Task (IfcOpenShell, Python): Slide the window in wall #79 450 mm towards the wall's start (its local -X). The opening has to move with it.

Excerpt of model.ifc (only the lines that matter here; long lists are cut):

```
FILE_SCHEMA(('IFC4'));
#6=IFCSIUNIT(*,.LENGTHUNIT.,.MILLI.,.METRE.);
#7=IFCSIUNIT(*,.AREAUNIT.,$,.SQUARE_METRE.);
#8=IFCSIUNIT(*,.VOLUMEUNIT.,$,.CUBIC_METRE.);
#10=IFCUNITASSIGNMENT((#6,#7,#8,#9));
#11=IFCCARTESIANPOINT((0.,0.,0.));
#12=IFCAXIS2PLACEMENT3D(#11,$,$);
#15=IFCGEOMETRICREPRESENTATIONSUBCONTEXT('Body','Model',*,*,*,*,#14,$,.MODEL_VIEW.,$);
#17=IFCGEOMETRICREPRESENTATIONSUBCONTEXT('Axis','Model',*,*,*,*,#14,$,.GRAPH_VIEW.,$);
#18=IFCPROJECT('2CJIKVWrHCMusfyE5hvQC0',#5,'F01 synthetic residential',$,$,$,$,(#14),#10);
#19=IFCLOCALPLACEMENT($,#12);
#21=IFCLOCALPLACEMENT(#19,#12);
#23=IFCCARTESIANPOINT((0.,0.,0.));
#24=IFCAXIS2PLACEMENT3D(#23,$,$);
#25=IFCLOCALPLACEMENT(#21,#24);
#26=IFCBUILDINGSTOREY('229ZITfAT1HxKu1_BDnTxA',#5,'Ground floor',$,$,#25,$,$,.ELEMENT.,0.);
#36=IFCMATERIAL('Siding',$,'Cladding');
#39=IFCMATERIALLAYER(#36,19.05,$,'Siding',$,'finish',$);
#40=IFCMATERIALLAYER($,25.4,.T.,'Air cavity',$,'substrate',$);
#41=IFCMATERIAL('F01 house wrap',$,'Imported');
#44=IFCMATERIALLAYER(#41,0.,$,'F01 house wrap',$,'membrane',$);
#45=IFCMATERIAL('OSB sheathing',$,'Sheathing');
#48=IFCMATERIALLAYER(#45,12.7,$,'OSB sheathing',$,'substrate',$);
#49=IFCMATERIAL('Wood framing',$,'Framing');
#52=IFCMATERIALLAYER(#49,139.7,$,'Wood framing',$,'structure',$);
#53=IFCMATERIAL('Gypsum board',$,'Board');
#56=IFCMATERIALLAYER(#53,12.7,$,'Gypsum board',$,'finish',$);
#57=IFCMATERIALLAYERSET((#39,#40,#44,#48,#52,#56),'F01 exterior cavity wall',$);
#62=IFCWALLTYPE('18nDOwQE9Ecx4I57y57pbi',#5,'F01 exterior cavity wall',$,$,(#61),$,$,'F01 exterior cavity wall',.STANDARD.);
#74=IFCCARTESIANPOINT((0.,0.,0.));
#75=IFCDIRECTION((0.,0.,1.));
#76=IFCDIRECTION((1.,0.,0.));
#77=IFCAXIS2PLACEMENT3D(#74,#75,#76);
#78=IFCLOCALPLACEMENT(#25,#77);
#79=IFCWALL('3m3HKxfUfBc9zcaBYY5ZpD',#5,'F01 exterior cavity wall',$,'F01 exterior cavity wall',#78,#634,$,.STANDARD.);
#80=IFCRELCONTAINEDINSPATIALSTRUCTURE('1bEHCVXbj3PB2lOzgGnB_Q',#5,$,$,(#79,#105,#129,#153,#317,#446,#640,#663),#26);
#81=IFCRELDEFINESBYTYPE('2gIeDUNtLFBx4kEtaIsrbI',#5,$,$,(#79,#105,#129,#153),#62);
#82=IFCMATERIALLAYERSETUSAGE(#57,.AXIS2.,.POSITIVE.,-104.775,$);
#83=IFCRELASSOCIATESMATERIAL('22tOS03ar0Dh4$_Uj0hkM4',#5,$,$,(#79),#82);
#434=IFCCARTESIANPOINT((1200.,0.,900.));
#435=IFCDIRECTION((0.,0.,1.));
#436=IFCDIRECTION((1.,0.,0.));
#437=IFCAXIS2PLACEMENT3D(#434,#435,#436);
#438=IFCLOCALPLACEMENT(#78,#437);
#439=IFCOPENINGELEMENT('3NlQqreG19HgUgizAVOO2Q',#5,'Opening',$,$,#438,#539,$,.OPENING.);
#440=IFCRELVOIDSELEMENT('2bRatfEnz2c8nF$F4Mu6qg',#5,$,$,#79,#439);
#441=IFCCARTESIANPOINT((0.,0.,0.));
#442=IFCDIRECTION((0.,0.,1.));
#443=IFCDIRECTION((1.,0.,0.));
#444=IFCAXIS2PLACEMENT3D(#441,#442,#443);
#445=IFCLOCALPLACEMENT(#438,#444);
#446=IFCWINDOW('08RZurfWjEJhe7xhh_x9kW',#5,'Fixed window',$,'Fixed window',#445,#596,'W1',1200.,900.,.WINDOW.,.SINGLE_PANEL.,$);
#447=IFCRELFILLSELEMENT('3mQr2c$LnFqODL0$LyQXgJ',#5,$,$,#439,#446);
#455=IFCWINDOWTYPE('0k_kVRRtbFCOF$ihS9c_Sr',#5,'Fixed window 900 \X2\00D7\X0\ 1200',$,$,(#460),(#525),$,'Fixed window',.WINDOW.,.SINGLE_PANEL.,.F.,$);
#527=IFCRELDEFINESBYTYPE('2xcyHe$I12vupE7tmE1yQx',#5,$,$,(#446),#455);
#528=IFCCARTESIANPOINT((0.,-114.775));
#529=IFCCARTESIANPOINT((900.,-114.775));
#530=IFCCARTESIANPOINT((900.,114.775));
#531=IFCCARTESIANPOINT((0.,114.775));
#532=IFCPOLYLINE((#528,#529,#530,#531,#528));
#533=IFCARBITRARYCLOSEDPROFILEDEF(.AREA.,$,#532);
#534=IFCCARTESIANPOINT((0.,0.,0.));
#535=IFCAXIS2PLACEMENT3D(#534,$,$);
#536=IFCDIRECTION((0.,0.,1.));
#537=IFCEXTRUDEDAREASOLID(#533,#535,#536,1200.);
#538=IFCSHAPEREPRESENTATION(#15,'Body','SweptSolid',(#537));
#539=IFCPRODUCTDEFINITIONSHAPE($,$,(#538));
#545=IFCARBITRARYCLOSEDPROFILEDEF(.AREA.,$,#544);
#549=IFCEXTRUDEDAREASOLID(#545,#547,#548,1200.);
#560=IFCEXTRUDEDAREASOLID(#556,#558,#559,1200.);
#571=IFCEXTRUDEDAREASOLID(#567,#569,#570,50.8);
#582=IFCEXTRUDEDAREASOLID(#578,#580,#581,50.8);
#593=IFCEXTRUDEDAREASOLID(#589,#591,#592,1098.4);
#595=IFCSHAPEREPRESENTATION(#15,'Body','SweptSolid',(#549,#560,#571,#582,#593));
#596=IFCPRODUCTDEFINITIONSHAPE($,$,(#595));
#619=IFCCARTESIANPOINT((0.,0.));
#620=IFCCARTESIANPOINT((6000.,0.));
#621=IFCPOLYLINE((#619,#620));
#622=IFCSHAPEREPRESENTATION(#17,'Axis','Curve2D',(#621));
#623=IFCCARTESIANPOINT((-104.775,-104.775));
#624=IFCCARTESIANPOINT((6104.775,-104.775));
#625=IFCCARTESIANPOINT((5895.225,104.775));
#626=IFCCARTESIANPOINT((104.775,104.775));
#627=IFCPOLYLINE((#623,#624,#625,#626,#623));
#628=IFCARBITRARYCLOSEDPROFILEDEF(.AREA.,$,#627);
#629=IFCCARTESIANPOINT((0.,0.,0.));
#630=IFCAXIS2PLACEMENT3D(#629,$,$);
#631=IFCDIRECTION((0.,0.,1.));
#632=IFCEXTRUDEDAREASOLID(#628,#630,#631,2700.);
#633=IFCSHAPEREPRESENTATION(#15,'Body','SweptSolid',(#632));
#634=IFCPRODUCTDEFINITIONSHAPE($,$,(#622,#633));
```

```python
import ifcopenshell
import ifcopenshell.api.geometry
import ifcopenshell.util.placement

model = ifcopenshell.open("model.ifc")

window = model.by_guid("08RZurfWjEJhe7xhh_x9kW")
opening = window.FillsVoids[0].RelatingOpeningElement
wall = opening.VoidsElements[0].RelatingBuildingElement

wall_matrix = ifcopenshell.util.placement.get_local_placement(wall.ObjectPlacement)
shift = wall_matrix[:3, 0] * -450.0
before = ifcopenshell.util.placement.get_local_placement(window.ObjectPlacement)[:3, 3].copy()

# The window is placed relative to its opening, so it follows when the opening moves.
matrix = ifcopenshell.util.placement.get_local_placement(opening.ObjectPlacement)
matrix[:3, 3] += shift
ifcopenshell.api.geometry.edit_object_placement(
    model, product=opening, matrix=matrix, is_si=False, should_transform_children=True
)

after = ifcopenshell.util.placement.get_local_placement(window.ObjectPlacement)[:3, 3]
print("window moved by", (after - before).round(3) + 0.0)

model.write("model_v2.ifc")
```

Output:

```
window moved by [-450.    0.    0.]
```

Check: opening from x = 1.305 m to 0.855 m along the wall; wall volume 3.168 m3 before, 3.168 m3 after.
